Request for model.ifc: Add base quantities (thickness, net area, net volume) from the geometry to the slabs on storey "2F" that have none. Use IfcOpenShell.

First a look at what the model holds.

```python
import ifcopenshell
import ifcopenshell.util.element
import ifcopenshell.util.unit

model = ifcopenshell.open("model.ifc")
print(model.schema)
for unit_type in ("LENGTHUNIT", "AREAUNIT", "VOLUMEUNIT"):
    print(unit_type, ifcopenshell.util.unit.calculate_unit_scale(model, unit_type))
storey = next(s for s in model.by_type("IfcBuildingStorey") if s.Name == "2F")
slabs = [e for e in ifcopenshell.util.element.get_decomposition(storey) if e.is_a("IfcSlab")]
for e in sorted(slabs, key=lambda e: e.id()):
    print(e.id(), e.is_a(), e.Name, list(ifcopenshell.util.element.get_psets(e, qtos_only=True)), sep=" | ")
```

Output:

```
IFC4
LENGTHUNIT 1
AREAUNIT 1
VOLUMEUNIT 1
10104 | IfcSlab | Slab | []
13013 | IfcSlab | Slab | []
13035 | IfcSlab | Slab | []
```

```python
import ifcopenshell
import ifcopenshell.api.pset
import ifcopenshell.geom
import ifcopenshell.util.element
import ifcopenshell.util.shape
import ifcopenshell.util.unit

model = ifcopenshell.open("model.ifc")
unit_scale = ifcopenshell.util.unit.calculate_unit_scale(model)
area_scale = ifcopenshell.util.unit.calculate_unit_scale(model, "AREAUNIT")
volume_scale = ifcopenshell.util.unit.calculate_unit_scale(model, "VOLUMEUNIT")
settings = ifcopenshell.geom.settings()

storey = next(s for s in model.by_type("IfcBuildingStorey") if s.Name == "2F")
slabs = [e for e in ifcopenshell.util.element.get_decomposition(storey) if e.is_a("IfcSlab")]

for e in sorted(slabs, key=lambda e: e.id()):
    if ifcopenshell.util.element.get_psets(e, qtos_only=True, should_inherit=False):
        continue
    # Geometry comes back in metres, in the element's own axes.
    shape = ifcopenshell.geom.create_shape(settings, e)
    values = {
        "Width": ifcopenshell.util.shape.get_z(shape.geometry) / unit_scale,
        "NetArea": ifcopenshell.util.shape.get_footprint_area(shape.geometry) / area_scale,
        "NetVolume": ifcopenshell.util.shape.get_volume(shape.geometry) / volume_scale,
    }
    qto = ifcopenshell.api.pset.add_qto(model, product=e, name="Qto_SlabBaseQuantities")
    ifcopenshell.api.pset.edit_qto(model, qto=qto, properties=values)
    print(e.id(), {k: round(v, 3) for k, v in values.items()})

model.write("model_edited.ifc")
```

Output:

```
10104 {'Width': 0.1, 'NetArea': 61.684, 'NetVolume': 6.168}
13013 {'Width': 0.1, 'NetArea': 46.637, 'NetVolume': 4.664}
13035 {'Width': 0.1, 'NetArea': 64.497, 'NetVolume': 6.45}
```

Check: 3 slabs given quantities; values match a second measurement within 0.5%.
